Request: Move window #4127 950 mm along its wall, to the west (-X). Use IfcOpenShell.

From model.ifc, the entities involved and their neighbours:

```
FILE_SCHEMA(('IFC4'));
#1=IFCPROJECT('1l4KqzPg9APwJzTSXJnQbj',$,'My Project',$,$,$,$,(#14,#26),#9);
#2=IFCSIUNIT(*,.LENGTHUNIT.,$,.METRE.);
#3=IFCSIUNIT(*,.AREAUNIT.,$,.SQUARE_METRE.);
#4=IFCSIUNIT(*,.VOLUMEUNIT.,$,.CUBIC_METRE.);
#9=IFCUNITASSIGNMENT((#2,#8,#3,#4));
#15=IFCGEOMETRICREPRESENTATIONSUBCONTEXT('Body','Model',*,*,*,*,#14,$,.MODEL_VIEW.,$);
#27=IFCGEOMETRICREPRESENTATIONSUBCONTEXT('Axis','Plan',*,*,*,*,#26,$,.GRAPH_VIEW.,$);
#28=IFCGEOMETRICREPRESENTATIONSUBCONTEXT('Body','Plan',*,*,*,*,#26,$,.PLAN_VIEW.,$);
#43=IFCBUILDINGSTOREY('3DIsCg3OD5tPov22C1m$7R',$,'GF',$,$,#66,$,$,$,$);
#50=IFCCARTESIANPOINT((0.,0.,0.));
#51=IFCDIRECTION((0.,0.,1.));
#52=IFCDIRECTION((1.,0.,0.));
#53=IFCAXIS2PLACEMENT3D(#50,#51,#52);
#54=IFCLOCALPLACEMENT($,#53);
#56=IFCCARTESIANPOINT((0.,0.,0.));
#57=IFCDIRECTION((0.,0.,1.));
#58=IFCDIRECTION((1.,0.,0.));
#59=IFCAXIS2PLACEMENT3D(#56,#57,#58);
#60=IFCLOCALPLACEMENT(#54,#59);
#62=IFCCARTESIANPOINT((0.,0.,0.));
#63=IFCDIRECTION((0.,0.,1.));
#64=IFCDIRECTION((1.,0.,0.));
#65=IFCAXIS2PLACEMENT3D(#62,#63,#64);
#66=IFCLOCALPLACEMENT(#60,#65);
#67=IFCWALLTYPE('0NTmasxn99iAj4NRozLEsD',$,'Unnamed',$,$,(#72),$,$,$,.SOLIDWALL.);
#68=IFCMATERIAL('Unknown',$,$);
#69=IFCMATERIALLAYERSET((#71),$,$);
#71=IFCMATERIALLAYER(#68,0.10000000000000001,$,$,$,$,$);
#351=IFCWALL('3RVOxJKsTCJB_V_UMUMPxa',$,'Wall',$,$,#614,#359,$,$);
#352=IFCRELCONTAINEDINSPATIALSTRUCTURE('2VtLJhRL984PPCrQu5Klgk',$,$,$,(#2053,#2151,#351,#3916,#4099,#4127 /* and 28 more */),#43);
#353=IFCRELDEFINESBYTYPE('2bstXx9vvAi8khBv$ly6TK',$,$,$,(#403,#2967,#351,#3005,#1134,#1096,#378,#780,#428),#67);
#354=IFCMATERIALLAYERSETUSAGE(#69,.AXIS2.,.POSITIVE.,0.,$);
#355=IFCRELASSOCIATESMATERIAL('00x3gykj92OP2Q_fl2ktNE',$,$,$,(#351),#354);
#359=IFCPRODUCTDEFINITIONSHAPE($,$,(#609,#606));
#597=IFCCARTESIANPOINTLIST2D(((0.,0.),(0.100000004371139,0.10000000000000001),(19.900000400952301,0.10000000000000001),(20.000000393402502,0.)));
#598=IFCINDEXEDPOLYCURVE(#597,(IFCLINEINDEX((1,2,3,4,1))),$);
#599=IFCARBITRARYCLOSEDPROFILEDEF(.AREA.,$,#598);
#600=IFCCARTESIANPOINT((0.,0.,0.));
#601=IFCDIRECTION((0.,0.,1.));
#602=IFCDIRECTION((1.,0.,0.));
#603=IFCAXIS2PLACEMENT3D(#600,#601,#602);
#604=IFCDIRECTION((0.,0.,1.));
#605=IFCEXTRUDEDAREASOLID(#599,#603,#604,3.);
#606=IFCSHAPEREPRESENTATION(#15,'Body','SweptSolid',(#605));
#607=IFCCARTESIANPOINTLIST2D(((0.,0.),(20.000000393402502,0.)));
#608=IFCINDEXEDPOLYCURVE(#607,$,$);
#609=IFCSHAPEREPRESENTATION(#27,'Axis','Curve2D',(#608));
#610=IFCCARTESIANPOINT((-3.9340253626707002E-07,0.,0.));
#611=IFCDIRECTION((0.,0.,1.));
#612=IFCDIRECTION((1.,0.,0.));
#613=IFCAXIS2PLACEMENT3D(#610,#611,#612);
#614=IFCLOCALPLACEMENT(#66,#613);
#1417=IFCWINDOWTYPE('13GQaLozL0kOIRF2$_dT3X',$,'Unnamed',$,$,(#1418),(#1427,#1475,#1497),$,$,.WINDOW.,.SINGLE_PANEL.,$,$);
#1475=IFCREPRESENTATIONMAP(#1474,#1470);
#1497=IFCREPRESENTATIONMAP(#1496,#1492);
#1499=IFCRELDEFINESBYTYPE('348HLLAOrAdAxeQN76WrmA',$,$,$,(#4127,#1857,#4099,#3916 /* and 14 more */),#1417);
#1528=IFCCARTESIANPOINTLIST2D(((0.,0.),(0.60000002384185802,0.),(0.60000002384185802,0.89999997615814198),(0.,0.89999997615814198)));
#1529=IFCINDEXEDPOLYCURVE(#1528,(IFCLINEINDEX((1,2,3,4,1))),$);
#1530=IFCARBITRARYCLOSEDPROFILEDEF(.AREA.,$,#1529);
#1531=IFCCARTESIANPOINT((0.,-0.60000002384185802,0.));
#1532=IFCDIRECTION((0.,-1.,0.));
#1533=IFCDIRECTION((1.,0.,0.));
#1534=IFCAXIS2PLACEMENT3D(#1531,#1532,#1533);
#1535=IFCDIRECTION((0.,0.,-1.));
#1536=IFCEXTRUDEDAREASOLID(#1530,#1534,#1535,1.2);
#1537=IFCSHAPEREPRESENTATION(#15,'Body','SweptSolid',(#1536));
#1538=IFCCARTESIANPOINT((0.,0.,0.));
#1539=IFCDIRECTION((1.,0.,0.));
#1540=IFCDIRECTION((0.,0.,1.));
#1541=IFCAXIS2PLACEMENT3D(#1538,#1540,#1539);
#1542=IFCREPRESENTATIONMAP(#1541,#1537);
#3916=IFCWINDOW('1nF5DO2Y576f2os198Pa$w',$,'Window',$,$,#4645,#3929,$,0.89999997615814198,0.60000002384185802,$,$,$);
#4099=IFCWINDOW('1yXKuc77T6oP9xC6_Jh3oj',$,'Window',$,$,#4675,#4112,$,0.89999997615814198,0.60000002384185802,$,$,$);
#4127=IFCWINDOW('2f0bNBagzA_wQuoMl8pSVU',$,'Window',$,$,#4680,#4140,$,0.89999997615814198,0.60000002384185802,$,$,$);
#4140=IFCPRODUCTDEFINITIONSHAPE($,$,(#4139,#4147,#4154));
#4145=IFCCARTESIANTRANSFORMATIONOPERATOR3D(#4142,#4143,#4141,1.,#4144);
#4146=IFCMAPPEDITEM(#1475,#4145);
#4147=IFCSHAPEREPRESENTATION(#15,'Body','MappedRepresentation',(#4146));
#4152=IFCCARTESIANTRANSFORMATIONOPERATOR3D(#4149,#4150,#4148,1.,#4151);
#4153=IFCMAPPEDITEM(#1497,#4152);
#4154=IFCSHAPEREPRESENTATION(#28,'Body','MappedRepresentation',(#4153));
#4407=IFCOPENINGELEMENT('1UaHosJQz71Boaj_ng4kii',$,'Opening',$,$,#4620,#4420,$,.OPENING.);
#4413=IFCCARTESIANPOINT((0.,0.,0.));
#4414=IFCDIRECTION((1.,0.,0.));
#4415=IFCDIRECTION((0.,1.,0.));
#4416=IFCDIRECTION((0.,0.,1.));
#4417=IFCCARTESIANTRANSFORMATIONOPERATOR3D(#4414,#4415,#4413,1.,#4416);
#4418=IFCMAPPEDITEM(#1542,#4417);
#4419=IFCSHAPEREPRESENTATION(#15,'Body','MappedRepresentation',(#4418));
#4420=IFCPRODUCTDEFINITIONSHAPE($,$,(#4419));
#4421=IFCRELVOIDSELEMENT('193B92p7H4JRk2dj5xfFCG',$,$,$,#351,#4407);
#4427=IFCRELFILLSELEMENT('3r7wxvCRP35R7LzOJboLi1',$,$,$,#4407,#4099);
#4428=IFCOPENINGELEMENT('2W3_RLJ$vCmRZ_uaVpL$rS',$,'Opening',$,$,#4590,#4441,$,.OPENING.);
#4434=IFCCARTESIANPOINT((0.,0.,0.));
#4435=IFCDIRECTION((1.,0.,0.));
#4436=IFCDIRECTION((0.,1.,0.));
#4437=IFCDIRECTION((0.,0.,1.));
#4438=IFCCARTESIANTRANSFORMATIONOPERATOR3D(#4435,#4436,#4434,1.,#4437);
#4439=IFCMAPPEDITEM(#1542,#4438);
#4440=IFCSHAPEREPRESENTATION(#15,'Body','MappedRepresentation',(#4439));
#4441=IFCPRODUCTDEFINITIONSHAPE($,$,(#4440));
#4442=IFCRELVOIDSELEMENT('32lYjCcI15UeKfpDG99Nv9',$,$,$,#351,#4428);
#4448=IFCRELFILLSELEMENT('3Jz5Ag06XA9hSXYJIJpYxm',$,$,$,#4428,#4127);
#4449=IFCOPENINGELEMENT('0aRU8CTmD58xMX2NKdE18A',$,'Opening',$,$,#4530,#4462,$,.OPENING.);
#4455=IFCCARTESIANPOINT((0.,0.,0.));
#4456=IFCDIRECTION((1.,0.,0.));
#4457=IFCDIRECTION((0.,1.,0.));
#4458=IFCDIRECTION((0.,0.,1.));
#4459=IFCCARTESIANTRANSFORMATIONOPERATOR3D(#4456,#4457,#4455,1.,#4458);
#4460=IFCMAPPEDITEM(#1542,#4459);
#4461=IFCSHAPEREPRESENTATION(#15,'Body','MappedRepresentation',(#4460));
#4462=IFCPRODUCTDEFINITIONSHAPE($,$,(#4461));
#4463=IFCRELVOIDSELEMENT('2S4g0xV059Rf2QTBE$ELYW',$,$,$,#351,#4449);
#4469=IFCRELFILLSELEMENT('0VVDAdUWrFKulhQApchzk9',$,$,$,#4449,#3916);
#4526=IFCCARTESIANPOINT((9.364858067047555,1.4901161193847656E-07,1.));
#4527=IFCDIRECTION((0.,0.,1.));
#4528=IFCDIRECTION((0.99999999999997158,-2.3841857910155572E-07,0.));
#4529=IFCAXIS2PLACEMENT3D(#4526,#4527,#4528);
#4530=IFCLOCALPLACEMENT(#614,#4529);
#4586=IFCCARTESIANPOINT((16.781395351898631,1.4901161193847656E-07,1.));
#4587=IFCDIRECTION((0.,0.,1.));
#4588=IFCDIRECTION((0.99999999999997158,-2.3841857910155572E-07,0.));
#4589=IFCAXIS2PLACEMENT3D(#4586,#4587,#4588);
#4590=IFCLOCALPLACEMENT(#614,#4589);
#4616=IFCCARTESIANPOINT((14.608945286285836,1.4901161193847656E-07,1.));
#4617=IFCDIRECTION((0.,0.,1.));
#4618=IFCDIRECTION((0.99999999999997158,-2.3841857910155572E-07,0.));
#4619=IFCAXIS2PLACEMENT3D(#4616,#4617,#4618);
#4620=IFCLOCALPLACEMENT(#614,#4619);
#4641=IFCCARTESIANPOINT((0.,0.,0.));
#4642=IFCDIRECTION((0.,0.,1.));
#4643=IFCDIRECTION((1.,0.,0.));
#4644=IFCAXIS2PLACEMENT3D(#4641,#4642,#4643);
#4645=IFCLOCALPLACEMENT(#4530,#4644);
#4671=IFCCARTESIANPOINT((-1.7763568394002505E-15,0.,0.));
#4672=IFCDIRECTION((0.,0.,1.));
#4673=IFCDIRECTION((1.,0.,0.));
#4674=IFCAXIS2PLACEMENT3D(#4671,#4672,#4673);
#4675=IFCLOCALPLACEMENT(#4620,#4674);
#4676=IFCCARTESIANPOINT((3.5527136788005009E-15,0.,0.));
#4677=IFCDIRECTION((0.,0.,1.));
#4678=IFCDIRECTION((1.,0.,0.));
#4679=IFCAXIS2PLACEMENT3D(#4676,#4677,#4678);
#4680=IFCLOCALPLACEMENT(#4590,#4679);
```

```python
import ifcopenshell
import ifcopenshell.api.geometry
import ifcopenshell.util.placement

model = ifcopenshell.open("model.ifc")

window = model.by_id(4127)
opening = window.FillsVoids[0].RelatingOpeningElement
wall = opening.VoidsElements[0].RelatingBuildingElement

wall_matrix = ifcopenshell.util.placement.get_local_placement(wall.ObjectPlacement)
shift = wall_matrix[:3, 0] * -0.95
before = ifcopenshell.util.placement.get_local_placement(window.ObjectPlacement)[:3, 3].copy()

# The window is placed relative to its opening, so it follows when the opening moves.
matrix = ifcopenshell.util.placement.get_local_placement(opening.ObjectPlacement)
matrix[:3, 3] += shift
ifcopenshell.api.geometry.edit_object_placement(
    model, product=opening, matrix=matrix, is_si=False, should_transform_children=True
)

after = ifcopenshell.util.placement.get_local_placement(window.ObjectPlacement)[:3, 3]
print("window moved by", (after - before).round(3) + 0.0)

model.write("model_v2.ifc")
```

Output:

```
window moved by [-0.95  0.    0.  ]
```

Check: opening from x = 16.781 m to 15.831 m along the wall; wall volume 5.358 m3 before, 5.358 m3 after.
